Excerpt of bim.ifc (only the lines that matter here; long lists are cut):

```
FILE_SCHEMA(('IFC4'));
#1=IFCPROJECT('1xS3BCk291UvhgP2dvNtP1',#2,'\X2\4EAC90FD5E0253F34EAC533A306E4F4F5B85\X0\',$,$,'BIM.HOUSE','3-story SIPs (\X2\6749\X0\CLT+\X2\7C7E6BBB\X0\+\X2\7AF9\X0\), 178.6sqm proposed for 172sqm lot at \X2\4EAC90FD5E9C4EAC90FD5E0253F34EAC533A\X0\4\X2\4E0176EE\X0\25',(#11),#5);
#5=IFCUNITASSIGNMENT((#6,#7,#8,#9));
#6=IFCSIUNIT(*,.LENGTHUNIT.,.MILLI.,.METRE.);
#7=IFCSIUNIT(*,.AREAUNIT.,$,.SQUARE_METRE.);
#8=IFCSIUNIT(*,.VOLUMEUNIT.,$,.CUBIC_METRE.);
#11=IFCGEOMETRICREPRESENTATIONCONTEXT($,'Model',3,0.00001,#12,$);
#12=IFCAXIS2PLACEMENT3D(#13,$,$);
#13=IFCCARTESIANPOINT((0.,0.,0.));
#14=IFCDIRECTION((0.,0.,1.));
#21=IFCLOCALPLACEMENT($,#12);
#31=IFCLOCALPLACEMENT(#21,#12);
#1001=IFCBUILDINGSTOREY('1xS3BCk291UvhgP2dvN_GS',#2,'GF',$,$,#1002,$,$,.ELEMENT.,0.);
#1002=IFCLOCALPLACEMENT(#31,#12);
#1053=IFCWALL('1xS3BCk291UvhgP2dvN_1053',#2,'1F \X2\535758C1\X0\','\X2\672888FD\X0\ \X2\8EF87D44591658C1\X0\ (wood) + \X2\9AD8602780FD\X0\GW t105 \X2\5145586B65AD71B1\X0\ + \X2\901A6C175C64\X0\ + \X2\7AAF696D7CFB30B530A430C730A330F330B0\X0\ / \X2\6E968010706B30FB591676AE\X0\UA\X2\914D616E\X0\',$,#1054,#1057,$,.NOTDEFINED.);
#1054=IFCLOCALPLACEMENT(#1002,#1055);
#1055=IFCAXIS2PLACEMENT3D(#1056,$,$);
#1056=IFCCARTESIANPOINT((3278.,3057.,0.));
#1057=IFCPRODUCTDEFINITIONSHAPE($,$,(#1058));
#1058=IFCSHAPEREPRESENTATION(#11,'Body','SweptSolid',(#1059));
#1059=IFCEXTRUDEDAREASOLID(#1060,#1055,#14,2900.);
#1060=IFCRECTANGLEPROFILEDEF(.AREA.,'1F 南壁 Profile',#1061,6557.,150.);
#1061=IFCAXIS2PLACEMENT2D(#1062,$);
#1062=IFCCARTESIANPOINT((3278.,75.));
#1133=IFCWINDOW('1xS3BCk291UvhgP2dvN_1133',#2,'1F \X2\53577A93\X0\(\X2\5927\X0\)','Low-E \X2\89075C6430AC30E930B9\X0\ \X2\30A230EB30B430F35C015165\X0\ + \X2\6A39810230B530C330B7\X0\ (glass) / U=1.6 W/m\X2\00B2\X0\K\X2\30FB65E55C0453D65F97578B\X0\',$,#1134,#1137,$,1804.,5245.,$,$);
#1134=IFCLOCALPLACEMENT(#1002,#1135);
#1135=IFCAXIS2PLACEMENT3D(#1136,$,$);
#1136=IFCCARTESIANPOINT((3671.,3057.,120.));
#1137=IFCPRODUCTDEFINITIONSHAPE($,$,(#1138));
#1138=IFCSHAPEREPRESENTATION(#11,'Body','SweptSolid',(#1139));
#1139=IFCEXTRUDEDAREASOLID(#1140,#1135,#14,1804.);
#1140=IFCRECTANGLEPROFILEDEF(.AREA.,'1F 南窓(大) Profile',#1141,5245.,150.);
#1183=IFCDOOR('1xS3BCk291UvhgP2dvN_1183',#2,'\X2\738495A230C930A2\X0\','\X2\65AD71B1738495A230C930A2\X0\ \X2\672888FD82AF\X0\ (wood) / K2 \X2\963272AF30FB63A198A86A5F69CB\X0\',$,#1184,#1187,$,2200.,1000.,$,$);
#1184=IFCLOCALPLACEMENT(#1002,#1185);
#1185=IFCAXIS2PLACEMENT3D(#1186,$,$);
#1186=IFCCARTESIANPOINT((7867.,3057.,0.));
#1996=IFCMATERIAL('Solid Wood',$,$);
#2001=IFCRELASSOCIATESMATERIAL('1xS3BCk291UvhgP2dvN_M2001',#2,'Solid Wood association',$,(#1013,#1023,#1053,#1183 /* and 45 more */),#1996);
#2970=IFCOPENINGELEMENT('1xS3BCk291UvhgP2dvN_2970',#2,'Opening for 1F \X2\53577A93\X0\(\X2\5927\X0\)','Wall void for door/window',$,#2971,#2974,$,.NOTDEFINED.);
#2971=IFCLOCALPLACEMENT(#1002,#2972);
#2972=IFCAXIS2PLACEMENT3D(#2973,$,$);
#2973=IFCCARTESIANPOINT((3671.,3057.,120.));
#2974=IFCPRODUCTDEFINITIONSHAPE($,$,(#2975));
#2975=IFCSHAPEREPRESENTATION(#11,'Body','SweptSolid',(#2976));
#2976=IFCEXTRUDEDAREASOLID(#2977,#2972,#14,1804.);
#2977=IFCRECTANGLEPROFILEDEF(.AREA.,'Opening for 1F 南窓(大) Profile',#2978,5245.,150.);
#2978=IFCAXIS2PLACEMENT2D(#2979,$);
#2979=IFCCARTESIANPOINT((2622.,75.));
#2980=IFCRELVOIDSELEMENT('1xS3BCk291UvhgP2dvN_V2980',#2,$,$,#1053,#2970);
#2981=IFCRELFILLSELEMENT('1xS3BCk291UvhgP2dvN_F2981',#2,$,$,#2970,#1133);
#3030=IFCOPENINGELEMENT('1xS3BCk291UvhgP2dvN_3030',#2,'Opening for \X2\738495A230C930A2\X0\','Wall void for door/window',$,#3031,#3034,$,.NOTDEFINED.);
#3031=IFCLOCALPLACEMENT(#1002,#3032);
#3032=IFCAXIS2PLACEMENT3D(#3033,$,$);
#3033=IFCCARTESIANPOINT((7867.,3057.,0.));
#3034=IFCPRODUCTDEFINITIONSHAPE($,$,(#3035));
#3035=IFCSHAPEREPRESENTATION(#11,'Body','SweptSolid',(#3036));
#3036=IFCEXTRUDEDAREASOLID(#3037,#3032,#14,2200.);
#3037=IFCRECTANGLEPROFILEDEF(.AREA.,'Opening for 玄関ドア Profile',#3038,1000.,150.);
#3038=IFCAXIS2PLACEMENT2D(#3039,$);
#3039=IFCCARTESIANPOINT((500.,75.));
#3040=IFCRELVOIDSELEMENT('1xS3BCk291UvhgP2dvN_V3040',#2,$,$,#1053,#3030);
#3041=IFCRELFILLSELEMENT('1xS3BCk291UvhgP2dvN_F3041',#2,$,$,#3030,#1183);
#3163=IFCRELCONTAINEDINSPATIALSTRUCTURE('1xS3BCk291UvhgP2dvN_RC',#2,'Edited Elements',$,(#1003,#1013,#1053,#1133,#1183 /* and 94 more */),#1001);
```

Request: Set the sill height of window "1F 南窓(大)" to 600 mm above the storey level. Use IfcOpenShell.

```python
import numpy as np
import ifcopenshell
import ifcopenshell.api.geometry
import ifcopenshell.geom
import ifcopenshell.util.element
import ifcopenshell.util.placement
import ifcopenshell.util.shape
import ifcopenshell.util.unit

model = ifcopenshell.open("bim.ifc")
unit_scale = ifcopenshell.util.unit.calculate_unit_scale(model)

window = model.by_guid("1xS3BCk291UvhgP2dvN_1133")
opening = window.FillsVoids[0].RelatingOpeningElement
storey = ifcopenshell.util.element.get_container(window, ifc_class="IfcBuildingStorey")
level = ifcopenshell.util.placement.get_local_placement(storey.ObjectPlacement)[2, 3]

# The opening's origin need not be at the sill, so measure its lowest point.
shape = ifcopenshell.geom.create_shape(ifcopenshell.geom.settings(), opening)
bottom = ifcopenshell.util.shape.get_shape_bottom_elevation(shape, shape.geometry) / unit_scale
dz = level + 0.6 / unit_scale - bottom

shift = np.array([0.0, 0.0, dz])
# The window is not placed relative to its opening, so move both.
for product in (opening, window):
    matrix = ifcopenshell.util.placement.get_local_placement(product.ObjectPlacement)
    matrix[:3, 3] += shift
    ifcopenshell.api.geometry.edit_object_placement(model, product=product, matrix=matrix, is_si=False)

print(f"moved by {dz * unit_scale:+.3f} m")

model.write("bim_rev.ifc")
```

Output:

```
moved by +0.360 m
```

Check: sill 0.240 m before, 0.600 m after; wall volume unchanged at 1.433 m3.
